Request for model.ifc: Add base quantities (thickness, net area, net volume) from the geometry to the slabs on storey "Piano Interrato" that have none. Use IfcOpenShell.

First a look at what the model holds.

```python
import ifcopenshell
import ifcopenshell.util.element
import ifcopenshell.util.unit

model = ifcopenshell.open("model.ifc")
print(model.schema)
for unit_type in ("LENGTHUNIT", "AREAUNIT", "VOLUMEUNIT"):
    print(unit_type, ifcopenshell.util.unit.calculate_unit_scale(model, unit_type))
storey = next(s for s in model.by_type("IfcBuildingStorey") if s.Name == "Piano Interrato")
slabs = [e for e in ifcopenshell.util.element.get_decomposition(storey) if e.is_a("IfcSlab")]
for e in sorted(slabs, key=lambda e: e.id()):
    print(e.id(), e.is_a(), e.Name, list(ifcopenshell.util.element.get_psets(e, qtos_only=True)), sep=" | ")
```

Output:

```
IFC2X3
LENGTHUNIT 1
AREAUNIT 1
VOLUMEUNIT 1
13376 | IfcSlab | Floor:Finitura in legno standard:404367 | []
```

```python
import ifcopenshell
import ifcopenshell.api.pset
import ifcopenshell.geom
import ifcopenshell.util.element
import ifcopenshell.util.shape
import ifcopenshell.util.unit

model = ifcopenshell.open("model.ifc")
unit_scale = ifcopenshell.util.unit.calculate_unit_scale(model)
area_scale = ifcopenshell.util.unit.calculate_unit_scale(model, "AREAUNIT")
volume_scale = ifcopenshell.util.unit.calculate_unit_scale(model, "VOLUMEUNIT")
settings = ifcopenshell.geom.settings()

storey = next(s for s in model.by_type("IfcBuildingStorey") if s.Name == "Piano Interrato")
slabs = [e for e in ifcopenshell.util.element.get_decomposition(storey) if e.is_a("IfcSlab")]

for e in sorted(slabs, key=lambda e: e.id()):
    if ifcopenshell.util.element.get_psets(e, qtos_only=True, should_inherit=False):
        continue
    # Geometry comes back in metres, in the element's own axes.
    shape = ifcopenshell.geom.create_shape(settings, e)
    values = {
        "Width": ifcopenshell.util.shape.get_z(shape.geometry) / unit_scale,
        "NetArea": ifcopenshell.util.shape.get_footprint_area(shape.geometry) / area_scale,
        "NetVolume": ifcopenshell.util.shape.get_volume(shape.geometry) / volume_scale,
    }
    qto = ifcopenshell.api.pset.add_qto(model, product=e, name="BaseQuantities")
    ifcopenshell.api.pset.edit_qto(model, qto=qto, properties=values)
    print(e.id(), {k: round(v, 3) for k, v in values.items()})

model.write("model_v2.ifc")
```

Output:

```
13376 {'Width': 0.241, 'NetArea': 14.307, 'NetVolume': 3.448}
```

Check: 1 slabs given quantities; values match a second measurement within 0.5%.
